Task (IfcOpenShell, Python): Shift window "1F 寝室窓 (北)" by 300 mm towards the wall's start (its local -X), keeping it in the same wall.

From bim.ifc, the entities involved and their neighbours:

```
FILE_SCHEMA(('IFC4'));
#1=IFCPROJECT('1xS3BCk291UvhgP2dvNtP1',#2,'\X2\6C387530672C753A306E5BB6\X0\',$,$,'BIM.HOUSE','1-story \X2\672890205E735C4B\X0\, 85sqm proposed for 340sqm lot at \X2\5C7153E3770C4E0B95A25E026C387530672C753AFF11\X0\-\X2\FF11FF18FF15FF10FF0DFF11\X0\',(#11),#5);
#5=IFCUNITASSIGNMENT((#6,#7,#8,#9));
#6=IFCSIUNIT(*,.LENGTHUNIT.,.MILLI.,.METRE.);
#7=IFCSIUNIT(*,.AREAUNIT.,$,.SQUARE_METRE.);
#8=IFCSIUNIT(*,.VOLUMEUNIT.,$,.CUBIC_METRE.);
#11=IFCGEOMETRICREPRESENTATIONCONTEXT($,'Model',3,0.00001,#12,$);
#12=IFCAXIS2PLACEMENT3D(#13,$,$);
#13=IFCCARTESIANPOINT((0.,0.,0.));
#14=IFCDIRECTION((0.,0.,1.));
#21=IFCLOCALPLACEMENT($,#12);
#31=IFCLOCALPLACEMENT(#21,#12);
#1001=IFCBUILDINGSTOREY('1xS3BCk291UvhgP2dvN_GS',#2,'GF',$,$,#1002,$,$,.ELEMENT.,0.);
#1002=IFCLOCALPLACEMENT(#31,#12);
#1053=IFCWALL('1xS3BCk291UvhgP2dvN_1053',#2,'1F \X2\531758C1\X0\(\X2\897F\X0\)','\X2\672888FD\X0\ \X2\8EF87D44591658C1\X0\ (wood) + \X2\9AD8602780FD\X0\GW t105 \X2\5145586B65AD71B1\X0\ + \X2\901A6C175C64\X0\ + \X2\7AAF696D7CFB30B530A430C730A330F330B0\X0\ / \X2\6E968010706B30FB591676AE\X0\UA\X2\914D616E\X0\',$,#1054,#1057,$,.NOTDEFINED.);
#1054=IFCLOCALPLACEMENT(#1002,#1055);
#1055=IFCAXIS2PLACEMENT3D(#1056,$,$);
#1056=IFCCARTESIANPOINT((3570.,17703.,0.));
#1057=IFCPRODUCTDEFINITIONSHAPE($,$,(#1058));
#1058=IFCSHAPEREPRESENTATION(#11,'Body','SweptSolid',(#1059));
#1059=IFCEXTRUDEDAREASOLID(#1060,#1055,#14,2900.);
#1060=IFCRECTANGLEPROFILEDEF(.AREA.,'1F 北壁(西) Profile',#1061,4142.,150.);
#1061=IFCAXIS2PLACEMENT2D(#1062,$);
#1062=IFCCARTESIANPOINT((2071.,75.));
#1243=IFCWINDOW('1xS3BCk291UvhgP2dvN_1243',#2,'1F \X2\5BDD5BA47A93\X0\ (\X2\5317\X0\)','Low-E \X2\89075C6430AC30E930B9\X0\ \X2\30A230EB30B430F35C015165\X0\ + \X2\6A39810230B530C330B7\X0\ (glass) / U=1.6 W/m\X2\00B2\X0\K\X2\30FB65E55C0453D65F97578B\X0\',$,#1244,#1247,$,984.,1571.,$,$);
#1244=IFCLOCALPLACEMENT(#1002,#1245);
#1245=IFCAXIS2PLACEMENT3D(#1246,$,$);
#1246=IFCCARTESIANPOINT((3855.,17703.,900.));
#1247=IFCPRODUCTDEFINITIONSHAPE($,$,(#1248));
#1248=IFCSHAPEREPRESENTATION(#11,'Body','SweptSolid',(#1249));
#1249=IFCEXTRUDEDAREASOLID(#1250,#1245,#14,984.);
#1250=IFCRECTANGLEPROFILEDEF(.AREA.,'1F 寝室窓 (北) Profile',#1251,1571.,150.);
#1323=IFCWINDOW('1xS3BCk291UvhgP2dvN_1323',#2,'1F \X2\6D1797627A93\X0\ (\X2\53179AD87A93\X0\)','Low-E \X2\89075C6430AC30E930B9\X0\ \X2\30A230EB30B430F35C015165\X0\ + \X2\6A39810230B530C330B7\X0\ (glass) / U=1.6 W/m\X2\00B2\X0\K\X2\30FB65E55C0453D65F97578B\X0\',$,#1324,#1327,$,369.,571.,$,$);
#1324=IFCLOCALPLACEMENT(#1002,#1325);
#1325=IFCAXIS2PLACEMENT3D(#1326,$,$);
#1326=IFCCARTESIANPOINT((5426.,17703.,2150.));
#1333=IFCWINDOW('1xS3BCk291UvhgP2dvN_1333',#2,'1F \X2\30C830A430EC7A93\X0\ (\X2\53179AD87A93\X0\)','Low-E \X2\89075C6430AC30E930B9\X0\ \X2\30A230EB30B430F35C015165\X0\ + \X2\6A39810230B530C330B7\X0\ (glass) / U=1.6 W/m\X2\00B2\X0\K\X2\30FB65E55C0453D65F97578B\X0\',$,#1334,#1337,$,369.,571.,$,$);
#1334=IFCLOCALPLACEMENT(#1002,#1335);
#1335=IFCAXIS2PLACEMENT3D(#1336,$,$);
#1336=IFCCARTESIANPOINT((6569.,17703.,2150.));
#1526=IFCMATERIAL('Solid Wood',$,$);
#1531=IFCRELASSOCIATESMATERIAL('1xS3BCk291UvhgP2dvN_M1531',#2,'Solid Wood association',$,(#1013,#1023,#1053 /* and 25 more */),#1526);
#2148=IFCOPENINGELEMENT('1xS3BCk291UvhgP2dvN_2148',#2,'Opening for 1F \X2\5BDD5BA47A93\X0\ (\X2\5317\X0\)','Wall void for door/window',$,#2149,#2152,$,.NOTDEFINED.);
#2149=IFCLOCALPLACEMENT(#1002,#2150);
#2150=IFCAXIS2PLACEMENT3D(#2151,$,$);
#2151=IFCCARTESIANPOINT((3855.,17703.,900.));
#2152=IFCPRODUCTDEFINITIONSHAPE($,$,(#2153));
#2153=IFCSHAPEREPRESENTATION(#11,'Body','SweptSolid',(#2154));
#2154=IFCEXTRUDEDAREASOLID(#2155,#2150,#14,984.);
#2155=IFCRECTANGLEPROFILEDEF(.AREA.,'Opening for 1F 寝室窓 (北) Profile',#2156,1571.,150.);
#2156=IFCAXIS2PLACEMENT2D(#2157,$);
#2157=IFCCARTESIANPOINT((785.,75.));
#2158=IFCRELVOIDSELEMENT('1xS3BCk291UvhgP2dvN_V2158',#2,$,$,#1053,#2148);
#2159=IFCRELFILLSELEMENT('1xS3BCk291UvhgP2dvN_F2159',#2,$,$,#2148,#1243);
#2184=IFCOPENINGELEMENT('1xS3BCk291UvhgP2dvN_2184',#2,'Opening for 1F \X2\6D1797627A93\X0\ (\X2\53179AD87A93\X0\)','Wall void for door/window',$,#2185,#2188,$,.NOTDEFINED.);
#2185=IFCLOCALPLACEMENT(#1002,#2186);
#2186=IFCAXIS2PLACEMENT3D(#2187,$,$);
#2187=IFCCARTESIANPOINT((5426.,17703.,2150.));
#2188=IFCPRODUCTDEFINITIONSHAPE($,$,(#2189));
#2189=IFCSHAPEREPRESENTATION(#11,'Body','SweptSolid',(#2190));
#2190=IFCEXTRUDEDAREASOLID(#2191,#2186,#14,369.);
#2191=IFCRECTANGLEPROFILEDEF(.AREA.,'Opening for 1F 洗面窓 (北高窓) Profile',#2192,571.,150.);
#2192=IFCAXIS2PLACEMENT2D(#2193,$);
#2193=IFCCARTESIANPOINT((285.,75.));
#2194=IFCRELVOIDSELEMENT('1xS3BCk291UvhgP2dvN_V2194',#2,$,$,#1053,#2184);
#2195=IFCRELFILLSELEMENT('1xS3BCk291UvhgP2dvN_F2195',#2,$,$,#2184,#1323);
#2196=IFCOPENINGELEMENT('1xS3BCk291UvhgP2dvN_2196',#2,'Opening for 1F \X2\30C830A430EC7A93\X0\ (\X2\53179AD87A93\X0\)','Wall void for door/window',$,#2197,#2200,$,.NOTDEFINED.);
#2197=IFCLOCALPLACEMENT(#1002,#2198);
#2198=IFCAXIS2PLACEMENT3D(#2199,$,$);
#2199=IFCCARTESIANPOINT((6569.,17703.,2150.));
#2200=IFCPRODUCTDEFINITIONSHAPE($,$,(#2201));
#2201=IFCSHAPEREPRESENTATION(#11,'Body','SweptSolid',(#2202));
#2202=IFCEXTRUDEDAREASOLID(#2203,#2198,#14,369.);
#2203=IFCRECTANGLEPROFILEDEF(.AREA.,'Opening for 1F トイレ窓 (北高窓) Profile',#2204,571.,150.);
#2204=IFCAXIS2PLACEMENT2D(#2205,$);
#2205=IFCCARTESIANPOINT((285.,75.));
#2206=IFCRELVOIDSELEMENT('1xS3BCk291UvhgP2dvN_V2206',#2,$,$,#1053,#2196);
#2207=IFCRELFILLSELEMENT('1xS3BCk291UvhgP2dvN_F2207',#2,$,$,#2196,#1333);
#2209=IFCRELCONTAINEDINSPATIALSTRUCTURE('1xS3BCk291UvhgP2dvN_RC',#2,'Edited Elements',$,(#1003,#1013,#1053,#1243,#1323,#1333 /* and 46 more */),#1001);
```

```python
import ifcopenshell
import ifcopenshell.api.geometry
import ifcopenshell.util.placement

model = ifcopenshell.open("bim.ifc")

window = model.by_guid("1xS3BCk291UvhgP2dvN_1243")
opening = window.FillsVoids[0].RelatingOpeningElement
wall = opening.VoidsElements[0].RelatingBuildingElement

wall_matrix = ifcopenshell.util.placement.get_local_placement(wall.ObjectPlacement)
shift = wall_matrix[:3, 0] * -300.0
before = ifcopenshell.util.placement.get_local_placement(window.ObjectPlacement)[:3, 3].copy()

# The window is not placed relative to its opening, so move both.
for product in (opening, window):
    matrix = ifcopenshell.util.placement.get_local_placement(product.ObjectPlacement)
    matrix[:3, 3] += shift
    ifcopenshell.api.geometry.edit_object_placement(model, product=product, matrix=matrix, is_si=False)

after = ifcopenshell.util.placement.get_local_placement(window.ObjectPlacement)[:3, 3]
print("window moved by", (after - before).round(3) + 0.0)

model.write("bim_updated.ifc")
```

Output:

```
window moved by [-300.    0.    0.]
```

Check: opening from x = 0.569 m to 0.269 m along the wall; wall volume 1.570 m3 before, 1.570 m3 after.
